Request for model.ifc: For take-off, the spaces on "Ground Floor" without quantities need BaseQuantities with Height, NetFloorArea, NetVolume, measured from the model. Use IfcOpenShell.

First a look at what the model holds.

```python
import ifcopenshell
import ifcopenshell.util.element
import ifcopenshell.util.unit

model = ifcopenshell.open("model.ifc")
print(model.schema)
for unit_type in ("LENGTHUNIT", "AREAUNIT", "VOLUMEUNIT"):
    print(unit_type, ifcopenshell.util.unit.calculate_unit_scale(model, unit_type))
storey = next(s for s in model.by_type("IfcBuildingStorey") if s.Name == "Ground Floor")
spaces = [e for e in ifcopenshell.util.element.get_decomposition(storey) if e.is_a("IfcSpace")]
for e in sorted(spaces, key=lambda e: e.id()):
    print(e.id(), e.is_a(), e.Name, list(ifcopenshell.util.element.get_psets(e, qtos_only=True)), sep=" | ")
```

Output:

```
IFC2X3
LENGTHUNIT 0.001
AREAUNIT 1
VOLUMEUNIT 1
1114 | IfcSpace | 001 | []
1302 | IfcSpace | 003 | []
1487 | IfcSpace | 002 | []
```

```python
import ifcopenshell
import ifcopenshell.api.pset
import ifcopenshell.geom
import ifcopenshell.util.element
import ifcopenshell.util.shape
import ifcopenshell.util.unit

model = ifcopenshell.open("model.ifc")
unit_scale = ifcopenshell.util.unit.calculate_unit_scale(model)
area_scale = ifcopenshell.util.unit.calculate_unit_scale(model, "AREAUNIT")
volume_scale = ifcopenshell.util.unit.calculate_unit_scale(model, "VOLUMEUNIT")
settings = ifcopenshell.geom.settings()

storey = next(s for s in model.by_type("IfcBuildingStorey") if s.Name == "Ground Floor")
spaces = [e for e in ifcopenshell.util.element.get_decomposition(storey) if e.is_a("IfcSpace")]

for e in sorted(spaces, key=lambda e: e.id()):
    if ifcopenshell.util.element.get_psets(e, qtos_only=True, should_inherit=False):
        continue
    # Geometry comes back in metres, in the element's own axes.
    shape = ifcopenshell.geom.create_shape(settings, e)
    values = {
        "Height": ifcopenshell.util.shape.get_z(shape.geometry) / unit_scale,
        "NetFloorArea": ifcopenshell.util.shape.get_footprint_area(shape.geometry) / area_scale,
        "NetVolume": ifcopenshell.util.shape.get_volume(shape.geometry) / volume_scale,
    }
    qto = ifcopenshell.api.pset.add_qto(model, product=e, name="BaseQuantities")
    ifcopenshell.api.pset.edit_qto(model, qto=qto, properties=values)
    print(e.id(), {k: round(v, 3) for k, v in values.items()})

model.write("model_rev.ifc")
```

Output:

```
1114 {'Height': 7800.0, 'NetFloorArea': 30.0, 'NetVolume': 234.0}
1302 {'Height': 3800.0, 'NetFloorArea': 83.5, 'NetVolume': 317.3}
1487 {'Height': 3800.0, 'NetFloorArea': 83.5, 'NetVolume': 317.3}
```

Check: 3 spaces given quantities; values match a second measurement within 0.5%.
